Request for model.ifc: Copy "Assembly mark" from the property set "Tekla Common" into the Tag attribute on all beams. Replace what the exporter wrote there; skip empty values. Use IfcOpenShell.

First a look at what the model holds.

```python
import ifcopenshell
import ifcopenshell.util.element

model = ifcopenshell.open("model.ifc")
print(model.schema)
beams = model.by_type("IfcBeam")
print(len(beams), "beams")
for e in beams[:8]:
    source = ifcopenshell.util.element.get_pset(e, "Tekla Common", "Assembly mark")
    target = e.Tag
    print(e.id(), repr(source), repr(target), sep=" | ")
```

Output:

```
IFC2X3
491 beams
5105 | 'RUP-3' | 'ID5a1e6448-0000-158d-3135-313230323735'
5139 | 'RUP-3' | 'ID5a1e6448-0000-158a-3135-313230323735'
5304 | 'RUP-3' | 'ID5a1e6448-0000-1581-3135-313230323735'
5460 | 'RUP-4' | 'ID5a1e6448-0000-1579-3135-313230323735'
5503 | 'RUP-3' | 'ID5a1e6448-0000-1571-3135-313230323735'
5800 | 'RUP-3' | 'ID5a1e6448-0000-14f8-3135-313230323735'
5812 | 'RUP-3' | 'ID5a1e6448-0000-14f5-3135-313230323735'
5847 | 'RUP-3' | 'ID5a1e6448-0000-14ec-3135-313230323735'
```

```python
import ifcopenshell
import ifcopenshell.util.element

model = ifcopenshell.open("model.ifc")

count = 0
for e in model.by_type("IfcBeam"):
    value = ifcopenshell.util.element.get_pset(e, "Tekla Common", "Assembly mark")
    current = e.Tag
    if not value or not value.strip() or current == value:
        continue
    e.Tag = value
    count += 1

print(count, "beams updated")

model.write("model_rev.ifc")
```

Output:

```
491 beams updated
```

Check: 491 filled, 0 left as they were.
